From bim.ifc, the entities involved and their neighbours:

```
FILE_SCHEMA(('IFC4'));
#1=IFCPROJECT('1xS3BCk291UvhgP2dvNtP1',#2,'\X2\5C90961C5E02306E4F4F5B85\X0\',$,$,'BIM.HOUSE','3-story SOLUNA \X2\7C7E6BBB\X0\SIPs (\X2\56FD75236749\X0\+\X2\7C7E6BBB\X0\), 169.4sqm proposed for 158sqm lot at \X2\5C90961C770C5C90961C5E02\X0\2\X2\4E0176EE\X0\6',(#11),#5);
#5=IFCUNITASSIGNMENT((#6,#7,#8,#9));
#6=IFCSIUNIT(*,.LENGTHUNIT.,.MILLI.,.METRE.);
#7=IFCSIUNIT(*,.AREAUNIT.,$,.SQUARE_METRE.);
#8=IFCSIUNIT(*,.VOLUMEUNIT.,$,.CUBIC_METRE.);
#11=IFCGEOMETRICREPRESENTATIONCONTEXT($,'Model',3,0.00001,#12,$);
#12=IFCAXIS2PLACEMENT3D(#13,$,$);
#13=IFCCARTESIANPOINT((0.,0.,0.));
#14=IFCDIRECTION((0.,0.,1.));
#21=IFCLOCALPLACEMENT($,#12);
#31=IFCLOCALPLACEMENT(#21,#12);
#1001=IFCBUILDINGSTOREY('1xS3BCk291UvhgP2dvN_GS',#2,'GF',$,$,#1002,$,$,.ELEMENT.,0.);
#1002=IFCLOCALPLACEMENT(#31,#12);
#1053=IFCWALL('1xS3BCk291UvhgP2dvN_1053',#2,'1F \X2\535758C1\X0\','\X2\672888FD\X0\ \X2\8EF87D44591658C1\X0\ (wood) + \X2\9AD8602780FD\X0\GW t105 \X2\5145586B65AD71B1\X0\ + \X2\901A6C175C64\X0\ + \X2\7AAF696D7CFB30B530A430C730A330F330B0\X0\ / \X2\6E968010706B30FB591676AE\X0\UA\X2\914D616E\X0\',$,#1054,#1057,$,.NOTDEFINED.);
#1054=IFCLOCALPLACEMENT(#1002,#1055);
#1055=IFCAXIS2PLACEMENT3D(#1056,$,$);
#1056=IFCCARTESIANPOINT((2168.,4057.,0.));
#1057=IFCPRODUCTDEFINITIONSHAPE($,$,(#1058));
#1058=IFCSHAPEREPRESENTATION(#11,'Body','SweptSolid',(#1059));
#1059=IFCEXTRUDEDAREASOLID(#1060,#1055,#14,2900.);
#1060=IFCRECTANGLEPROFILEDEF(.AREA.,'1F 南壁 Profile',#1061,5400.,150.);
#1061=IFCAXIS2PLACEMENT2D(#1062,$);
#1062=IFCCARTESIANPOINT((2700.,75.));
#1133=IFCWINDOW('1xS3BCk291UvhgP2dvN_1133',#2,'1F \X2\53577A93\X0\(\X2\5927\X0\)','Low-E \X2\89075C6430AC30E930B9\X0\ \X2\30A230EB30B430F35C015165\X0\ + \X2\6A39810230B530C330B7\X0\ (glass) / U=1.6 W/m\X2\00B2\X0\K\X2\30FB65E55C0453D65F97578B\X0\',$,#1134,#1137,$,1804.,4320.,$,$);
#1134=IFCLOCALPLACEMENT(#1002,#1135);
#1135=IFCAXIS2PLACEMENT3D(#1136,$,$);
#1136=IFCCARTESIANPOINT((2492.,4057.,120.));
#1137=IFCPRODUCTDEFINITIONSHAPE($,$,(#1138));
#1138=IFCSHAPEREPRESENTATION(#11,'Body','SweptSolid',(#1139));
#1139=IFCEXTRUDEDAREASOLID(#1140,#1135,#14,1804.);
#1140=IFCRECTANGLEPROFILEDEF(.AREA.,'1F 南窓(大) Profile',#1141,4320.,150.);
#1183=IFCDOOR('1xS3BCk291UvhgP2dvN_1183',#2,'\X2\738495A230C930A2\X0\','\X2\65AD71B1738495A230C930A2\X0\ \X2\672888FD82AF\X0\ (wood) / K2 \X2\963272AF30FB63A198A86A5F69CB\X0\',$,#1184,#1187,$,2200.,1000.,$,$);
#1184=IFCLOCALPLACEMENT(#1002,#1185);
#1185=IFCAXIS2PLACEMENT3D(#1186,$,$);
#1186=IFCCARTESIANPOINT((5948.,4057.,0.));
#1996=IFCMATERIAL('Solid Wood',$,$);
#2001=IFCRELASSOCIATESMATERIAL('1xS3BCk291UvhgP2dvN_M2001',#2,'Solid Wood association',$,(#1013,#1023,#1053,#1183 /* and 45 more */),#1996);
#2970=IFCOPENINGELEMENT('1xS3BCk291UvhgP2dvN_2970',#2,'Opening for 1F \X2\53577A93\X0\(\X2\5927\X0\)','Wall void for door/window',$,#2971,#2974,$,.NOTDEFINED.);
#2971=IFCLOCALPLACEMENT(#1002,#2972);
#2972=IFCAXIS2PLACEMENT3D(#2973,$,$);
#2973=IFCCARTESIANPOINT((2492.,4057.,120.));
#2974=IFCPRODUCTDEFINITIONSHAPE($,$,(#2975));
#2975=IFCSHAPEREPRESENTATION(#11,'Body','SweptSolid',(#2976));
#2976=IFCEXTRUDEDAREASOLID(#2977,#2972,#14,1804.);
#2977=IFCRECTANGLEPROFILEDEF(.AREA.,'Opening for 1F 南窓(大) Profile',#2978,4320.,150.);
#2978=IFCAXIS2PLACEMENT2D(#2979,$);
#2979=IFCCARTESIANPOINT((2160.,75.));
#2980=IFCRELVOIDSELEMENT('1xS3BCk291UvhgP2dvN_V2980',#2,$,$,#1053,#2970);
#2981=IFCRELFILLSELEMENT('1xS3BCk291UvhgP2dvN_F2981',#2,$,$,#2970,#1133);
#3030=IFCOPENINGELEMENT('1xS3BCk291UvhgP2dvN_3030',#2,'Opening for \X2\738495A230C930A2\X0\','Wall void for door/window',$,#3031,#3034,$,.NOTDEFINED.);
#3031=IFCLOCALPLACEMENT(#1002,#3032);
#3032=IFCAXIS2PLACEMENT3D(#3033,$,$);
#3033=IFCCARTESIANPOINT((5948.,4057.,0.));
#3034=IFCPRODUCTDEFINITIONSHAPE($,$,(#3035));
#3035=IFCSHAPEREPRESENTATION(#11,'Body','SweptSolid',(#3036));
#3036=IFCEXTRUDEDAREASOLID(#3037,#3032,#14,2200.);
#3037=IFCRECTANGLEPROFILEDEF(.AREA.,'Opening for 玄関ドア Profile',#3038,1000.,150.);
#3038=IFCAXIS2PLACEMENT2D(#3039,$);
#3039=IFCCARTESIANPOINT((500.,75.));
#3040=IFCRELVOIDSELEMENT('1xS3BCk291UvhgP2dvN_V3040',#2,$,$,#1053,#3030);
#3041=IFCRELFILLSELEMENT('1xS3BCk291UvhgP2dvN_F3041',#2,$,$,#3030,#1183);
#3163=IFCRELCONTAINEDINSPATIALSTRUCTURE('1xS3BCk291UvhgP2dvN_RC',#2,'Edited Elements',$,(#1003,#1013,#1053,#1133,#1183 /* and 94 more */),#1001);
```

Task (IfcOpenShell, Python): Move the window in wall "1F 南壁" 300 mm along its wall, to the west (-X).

```python
import ifcopenshell
import ifcopenshell.api.geometry
import ifcopenshell.util.placement
import ifcopenshell.util.unit

model = ifcopenshell.open("bim.ifc")
unit_scale = ifcopenshell.util.unit.calculate_unit_scale(model)

window = model.by_guid("1xS3BCk291UvhgP2dvN_1133")
opening = window.FillsVoids[0].RelatingOpeningElement
wall = opening.VoidsElements[0].RelatingBuildingElement

wall_matrix = ifcopenshell.util.placement.get_local_placement(wall.ObjectPlacement)
shift = wall_matrix[:3, 0] * -0.3 / unit_scale
before = ifcopenshell.util.placement.get_local_placement(window.ObjectPlacement)[:3, 3].copy()

# The window is not placed relative to its opening, so move both.
for product in (opening, window):
    matrix = ifcopenshell.util.placement.get_local_placement(product.ObjectPlacement)
    matrix[:3, 3] += shift
    ifcopenshell.api.geometry.edit_object_placement(model, product=product, matrix=matrix, is_si=False)

after = ifcopenshell.util.placement.get_local_placement(window.ObjectPlacement)[:3, 3]
print("window moved by", (after - before).round(3) + 0.0)

model.write("bim-out.ifc")
```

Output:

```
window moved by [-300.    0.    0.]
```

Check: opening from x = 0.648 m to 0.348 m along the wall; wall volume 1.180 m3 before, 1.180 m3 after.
